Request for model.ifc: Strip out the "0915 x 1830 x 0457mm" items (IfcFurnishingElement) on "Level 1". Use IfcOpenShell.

First a look at what the model holds.

```python
import ifcopenshell
import ifcopenshell.util.element

model = ifcopenshell.open("model.ifc")
print(model.schema)
storey = next(s for s in model.by_type("IfcBuildingStorey") if s.Name == "Level 1")
furniture = [e for e in ifcopenshell.util.element.get_decomposition(storey) if e.is_a("IfcFurnishingElement")]
seen = {}
for e in furniture:
    element_type = ifcopenshell.util.element.get_type(e)
    name = element_type.Name if element_type not in (None, e) else None
    seen[name] = seen.get(name, 0) + 1
for name, count in sorted(seen.items(), key=str):
    print(count, "x", name)
```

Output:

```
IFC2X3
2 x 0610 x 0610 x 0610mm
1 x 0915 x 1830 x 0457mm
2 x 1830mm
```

```python
import ifcopenshell
import ifcopenshell.api.root
import ifcopenshell.util.element

model = ifcopenshell.open("model.ifc")

storey = next(s for s in model.by_type("IfcBuildingStorey") if s.Name == "Level 1")
furniture = [e for e in ifcopenshell.util.element.get_decomposition(storey) if e.is_a("IfcFurnishingElement")]
targets = [e for e in furniture if (t := ifcopenshell.util.element.get_type(e)) not in (None, e) and t.Name == "0915 x 1830 x 0457mm"]

for e in targets:
    ifcopenshell.api.root.remove_product(model, product=e)
print(len(targets), "removed")

model.write("model_rev.ifc")
```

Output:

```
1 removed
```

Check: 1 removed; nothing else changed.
